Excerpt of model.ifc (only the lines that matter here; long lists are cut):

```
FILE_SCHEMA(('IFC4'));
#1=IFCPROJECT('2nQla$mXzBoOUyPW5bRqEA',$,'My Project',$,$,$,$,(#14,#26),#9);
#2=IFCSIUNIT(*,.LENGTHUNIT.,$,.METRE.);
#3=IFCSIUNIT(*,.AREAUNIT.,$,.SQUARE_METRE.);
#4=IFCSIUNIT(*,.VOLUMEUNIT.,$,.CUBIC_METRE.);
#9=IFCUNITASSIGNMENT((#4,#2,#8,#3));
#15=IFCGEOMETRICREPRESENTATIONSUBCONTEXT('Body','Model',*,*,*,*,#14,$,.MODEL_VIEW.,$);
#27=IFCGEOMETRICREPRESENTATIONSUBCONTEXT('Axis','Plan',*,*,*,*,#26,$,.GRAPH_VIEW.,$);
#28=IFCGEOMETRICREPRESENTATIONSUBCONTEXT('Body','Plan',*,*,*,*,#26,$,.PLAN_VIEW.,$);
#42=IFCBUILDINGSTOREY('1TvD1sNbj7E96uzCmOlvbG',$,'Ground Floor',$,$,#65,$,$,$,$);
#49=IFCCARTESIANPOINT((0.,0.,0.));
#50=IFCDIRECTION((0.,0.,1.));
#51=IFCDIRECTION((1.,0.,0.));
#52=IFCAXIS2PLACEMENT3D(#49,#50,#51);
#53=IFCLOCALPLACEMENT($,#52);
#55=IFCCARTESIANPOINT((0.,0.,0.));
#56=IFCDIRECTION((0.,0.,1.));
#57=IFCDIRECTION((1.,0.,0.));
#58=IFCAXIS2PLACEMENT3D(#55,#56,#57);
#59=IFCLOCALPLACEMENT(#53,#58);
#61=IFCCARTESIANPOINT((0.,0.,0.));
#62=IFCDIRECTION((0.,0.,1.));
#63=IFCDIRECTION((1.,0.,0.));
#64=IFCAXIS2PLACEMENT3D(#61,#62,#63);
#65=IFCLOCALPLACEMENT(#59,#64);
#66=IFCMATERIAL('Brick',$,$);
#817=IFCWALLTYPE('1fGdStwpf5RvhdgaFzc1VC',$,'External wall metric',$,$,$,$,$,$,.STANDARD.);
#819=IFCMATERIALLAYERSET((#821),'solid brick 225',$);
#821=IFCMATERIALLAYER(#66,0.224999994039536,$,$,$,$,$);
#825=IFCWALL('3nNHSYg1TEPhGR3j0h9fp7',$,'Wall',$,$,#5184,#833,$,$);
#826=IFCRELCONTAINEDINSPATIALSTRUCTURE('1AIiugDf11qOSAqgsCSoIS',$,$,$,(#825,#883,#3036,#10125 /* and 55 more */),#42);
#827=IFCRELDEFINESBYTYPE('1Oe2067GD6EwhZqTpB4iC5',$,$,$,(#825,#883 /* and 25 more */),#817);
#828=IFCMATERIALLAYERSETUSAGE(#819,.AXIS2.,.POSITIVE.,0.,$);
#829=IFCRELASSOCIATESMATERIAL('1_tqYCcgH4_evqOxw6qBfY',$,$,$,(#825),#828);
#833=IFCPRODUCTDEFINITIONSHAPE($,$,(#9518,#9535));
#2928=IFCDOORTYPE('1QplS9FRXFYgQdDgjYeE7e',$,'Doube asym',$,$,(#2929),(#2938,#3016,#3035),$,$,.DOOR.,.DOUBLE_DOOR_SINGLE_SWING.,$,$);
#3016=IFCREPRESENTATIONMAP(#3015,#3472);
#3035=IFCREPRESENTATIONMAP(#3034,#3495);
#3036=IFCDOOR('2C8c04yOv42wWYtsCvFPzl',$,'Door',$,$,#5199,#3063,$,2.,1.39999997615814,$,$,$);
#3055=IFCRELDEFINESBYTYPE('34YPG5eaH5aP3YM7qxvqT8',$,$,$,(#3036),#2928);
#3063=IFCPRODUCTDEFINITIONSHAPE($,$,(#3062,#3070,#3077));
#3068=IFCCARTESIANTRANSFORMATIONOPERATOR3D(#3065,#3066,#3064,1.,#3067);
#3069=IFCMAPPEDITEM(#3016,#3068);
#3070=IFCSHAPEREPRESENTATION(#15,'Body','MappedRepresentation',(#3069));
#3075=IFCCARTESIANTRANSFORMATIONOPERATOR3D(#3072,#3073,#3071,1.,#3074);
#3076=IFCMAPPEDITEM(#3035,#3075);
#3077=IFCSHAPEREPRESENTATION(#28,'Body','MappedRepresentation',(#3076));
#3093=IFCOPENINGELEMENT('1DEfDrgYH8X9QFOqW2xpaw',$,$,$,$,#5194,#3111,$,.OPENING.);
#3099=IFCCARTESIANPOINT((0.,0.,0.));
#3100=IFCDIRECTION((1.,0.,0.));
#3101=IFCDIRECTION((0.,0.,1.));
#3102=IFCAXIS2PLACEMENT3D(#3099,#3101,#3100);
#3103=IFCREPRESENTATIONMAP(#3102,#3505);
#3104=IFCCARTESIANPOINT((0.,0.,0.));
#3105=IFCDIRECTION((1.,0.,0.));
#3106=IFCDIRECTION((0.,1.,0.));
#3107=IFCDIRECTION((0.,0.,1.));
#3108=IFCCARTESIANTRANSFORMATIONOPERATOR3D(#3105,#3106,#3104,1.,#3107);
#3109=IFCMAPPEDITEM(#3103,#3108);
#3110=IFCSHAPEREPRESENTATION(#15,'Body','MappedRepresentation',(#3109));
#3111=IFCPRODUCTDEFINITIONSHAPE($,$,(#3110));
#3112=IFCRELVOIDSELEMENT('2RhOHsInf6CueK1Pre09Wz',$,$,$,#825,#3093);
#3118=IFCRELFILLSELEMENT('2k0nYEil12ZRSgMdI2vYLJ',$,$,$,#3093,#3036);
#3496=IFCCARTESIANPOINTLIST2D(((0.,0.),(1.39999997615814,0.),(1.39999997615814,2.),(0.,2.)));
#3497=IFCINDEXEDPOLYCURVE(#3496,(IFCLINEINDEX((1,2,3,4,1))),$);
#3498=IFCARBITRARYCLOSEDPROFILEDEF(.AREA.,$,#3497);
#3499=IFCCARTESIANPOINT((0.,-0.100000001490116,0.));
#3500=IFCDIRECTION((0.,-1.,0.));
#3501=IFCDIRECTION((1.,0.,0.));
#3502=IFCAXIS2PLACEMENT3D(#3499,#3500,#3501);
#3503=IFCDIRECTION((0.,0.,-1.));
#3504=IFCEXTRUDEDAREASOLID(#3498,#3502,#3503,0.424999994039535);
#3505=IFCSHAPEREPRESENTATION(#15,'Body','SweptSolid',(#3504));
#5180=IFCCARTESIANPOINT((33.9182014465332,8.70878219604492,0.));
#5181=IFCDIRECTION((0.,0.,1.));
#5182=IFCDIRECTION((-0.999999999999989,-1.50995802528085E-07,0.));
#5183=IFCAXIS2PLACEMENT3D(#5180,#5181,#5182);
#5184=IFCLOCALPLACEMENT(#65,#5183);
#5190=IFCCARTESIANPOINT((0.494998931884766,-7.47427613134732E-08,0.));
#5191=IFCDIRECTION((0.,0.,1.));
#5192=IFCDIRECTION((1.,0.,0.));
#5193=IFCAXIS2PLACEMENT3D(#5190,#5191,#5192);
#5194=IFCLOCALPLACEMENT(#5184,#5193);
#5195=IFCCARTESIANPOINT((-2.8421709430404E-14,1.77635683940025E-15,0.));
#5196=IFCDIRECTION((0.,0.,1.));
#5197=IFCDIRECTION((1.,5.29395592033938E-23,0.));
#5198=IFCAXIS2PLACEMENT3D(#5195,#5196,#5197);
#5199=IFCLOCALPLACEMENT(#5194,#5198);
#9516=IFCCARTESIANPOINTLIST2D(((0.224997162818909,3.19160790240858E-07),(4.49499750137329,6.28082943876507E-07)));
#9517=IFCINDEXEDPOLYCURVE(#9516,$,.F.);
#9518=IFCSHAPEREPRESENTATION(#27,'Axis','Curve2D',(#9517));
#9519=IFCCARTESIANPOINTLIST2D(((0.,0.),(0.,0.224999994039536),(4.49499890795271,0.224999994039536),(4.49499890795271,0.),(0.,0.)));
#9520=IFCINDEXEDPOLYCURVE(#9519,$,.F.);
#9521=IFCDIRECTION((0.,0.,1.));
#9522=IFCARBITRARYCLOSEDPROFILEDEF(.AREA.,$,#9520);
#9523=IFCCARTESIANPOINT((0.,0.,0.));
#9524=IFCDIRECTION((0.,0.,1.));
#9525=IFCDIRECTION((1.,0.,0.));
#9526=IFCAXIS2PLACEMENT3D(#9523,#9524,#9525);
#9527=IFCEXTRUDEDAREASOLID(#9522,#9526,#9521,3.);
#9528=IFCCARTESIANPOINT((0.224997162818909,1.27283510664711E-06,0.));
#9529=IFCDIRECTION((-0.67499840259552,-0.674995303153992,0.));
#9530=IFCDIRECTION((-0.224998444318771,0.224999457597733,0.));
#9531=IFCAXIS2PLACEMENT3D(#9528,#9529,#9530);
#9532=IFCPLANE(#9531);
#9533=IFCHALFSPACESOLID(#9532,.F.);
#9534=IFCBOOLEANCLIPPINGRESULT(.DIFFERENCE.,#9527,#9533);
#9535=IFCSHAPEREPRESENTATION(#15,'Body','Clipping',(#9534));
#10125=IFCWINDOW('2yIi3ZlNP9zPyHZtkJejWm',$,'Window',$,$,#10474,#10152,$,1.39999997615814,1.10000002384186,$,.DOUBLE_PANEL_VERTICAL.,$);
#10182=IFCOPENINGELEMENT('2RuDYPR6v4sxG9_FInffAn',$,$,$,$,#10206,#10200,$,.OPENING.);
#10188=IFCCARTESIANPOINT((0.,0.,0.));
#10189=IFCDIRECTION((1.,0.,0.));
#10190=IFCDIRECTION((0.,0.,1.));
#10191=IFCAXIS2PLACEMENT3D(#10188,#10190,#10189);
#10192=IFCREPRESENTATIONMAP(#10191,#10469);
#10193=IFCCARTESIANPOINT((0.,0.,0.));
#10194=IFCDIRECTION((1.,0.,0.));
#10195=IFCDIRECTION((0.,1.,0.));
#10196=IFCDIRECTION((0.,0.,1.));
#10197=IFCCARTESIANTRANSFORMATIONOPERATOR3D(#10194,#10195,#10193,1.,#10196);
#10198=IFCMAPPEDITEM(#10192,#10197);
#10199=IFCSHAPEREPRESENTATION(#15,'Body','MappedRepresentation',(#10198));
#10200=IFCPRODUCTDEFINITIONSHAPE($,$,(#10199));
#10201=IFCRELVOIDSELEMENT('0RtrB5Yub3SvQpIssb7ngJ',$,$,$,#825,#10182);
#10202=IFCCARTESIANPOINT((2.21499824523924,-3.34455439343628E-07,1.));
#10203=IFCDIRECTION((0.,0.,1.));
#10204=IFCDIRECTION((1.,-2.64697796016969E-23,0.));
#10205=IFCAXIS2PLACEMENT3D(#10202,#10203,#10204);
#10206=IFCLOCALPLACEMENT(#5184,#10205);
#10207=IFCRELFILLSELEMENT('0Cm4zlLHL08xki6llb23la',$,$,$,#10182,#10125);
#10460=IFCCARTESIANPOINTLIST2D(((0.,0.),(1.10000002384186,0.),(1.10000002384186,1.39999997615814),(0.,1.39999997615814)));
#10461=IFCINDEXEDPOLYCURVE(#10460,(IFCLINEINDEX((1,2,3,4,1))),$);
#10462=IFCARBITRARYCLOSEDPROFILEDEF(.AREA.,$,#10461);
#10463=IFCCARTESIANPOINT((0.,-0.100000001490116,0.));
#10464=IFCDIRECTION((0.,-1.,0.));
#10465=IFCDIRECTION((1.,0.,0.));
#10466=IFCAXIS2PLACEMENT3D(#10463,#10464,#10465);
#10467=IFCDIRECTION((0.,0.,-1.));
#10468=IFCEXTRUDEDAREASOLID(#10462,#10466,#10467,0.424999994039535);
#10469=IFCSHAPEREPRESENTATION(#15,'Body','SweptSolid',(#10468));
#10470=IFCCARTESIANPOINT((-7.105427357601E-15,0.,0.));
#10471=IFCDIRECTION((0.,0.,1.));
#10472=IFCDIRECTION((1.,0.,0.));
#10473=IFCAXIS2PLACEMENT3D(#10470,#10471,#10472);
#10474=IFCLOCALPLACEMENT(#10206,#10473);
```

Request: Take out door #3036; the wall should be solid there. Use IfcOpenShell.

```python
import ifcopenshell
import ifcopenshell.api.feature
import ifcopenshell.api.root
import ifcopenshell.geom
import ifcopenshell.util.shape

model = ifcopenshell.open("model.ifc")
settings = ifcopenshell.geom.settings()


def volume(element):
    """Net volume in cubic metres, openings subtracted."""
    shape = ifcopenshell.geom.create_shape(settings, element)
    return ifcopenshell.util.shape.get_volume(shape.geometry)


door = model.by_guid("2C8c04yOv42wWYtsCvFPzl")
opening = door.FillsVoids[0].RelatingOpeningElement
wall = opening.VoidsElements[0].RelatingBuildingElement
before = volume(wall)

ifcopenshell.api.root.remove_product(model, product=door)
ifcopenshell.api.feature.remove_feature(model, feature=opening)

after = volume(wall)

print(f"wall volume {before:.3f} -> {after:.3f} m3")

model.write("model_updated.ifc")
```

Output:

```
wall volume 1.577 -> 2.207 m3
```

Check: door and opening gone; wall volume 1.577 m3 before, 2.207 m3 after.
